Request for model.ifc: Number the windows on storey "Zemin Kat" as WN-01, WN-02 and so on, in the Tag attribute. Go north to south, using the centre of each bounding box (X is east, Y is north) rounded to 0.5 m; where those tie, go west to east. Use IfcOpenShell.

First a look at what the model holds.

```python
import ifcopenshell
import ifcopenshell.util.element
import ifcopenshell.util.placement

model = ifcopenshell.open("model.ifc")
print(model.schema)
storey = next(s for s in model.by_type("IfcBuildingStorey") if s.Name == "Zemin Kat")
windows = [e for e in ifcopenshell.util.element.get_decomposition(storey) if e.is_a("IfcWindow")]
for e in sorted(windows, key=lambda e: e.id()):
    origin = ifcopenshell.util.placement.get_local_placement(e.ObjectPlacement)[:3, 3]
    print(e.id(), e.Tag, e.Name, origin.round(2) + 0.0, sep=" | ")
```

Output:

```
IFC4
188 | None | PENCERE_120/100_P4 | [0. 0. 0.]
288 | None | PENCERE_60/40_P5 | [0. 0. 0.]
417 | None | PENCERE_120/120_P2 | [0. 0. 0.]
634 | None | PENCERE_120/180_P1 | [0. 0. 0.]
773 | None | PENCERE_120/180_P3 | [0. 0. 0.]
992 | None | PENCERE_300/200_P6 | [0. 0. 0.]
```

```python
import ifcopenshell
import ifcopenshell.geom
import ifcopenshell.util.element
import ifcopenshell.util.shape

model = ifcopenshell.open("model.ifc")
settings = ifcopenshell.geom.settings()
settings.set("use-world-coords", True)


def centre(element):
    shape = ifcopenshell.geom.create_shape(settings, element)
    return ifcopenshell.util.shape.get_bbox_centroid(shape.geometry)


storey = next(s for s in model.by_type("IfcBuildingStorey") if s.Name == "Zemin Kat")
windows = [e for e in ifcopenshell.util.element.get_decomposition(storey) if e.is_a("IfcWindow")]

# Insertion points can sit at a corner or the storey origin, so sort by the geometry (in metres).
centres = {e: centre(e) for e in windows}
windows.sort(key=lambda e: (-round(centres[e][1] / 0.5), centres[e][0]))

for i, e in enumerate(windows, start=1):
    number = f"WN-{i:02d}"
    e.Tag = number
    print(e.id(), number)

model.write("model_updated.ifc")
```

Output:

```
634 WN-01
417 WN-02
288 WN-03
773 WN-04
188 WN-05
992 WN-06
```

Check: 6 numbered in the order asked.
